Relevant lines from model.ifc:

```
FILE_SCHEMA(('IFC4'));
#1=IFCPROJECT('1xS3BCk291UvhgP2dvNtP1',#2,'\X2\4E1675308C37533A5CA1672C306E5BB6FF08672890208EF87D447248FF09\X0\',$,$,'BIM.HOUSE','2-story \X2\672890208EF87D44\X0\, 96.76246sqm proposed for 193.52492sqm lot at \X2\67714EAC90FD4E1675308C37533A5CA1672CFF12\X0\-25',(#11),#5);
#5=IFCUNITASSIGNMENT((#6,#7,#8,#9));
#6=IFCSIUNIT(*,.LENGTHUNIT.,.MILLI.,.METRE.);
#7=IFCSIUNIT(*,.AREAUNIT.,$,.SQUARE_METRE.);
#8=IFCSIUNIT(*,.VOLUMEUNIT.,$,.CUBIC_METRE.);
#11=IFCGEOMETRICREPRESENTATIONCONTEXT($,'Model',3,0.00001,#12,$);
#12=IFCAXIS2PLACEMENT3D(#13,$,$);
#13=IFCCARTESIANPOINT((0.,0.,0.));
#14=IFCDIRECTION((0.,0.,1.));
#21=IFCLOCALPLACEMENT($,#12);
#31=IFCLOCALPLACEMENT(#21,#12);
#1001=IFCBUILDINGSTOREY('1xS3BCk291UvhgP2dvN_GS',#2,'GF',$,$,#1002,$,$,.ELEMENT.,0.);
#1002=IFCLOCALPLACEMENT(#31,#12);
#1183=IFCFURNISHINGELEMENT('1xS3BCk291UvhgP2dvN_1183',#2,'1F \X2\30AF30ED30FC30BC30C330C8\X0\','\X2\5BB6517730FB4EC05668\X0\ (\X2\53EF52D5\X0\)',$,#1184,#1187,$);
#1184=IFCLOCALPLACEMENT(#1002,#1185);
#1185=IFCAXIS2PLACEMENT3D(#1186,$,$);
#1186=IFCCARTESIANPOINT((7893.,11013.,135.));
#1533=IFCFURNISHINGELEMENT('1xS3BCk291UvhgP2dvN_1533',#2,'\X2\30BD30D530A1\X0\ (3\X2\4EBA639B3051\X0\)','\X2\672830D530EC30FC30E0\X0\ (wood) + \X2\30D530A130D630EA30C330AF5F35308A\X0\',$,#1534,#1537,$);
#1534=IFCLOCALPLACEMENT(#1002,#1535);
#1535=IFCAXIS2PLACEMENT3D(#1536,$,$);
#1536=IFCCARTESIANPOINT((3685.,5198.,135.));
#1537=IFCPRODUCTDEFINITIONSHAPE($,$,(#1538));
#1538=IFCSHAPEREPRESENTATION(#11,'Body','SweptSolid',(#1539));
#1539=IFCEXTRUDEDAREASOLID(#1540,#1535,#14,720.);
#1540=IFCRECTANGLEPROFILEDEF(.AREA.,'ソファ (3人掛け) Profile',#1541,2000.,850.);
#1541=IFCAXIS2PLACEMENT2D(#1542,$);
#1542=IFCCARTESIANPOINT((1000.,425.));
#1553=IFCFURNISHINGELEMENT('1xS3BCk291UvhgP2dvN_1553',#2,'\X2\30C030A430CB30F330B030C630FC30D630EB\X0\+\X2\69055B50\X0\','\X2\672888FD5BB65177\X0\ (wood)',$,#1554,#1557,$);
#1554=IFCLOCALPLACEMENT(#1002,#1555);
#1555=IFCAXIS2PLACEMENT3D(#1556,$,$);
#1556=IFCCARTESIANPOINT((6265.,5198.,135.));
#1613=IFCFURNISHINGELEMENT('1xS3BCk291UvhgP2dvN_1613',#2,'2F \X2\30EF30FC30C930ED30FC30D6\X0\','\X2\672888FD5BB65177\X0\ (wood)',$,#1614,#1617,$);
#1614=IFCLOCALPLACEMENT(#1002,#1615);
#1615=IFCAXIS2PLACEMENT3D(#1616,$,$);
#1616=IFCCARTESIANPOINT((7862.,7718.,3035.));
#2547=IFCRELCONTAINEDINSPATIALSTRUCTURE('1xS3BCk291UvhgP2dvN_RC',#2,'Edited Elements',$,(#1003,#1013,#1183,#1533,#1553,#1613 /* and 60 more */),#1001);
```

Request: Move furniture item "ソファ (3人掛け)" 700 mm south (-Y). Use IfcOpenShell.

```python
import ifcopenshell
import ifcopenshell.api.geometry
import ifcopenshell.util.placement

model = ifcopenshell.open("model.ifc")

item = model.by_guid("1xS3BCk291UvhgP2dvN_1533")
matrix = ifcopenshell.util.placement.get_local_placement(item.ObjectPlacement)
matrix[1, 3] -= 700.0
ifcopenshell.api.geometry.edit_object_placement(model, product=item, matrix=matrix, is_si=False)

print(ifcopenshell.util.placement.get_local_placement(item.ObjectPlacement).round(3) + 0.0)

model.write("model_edited.ifc")
```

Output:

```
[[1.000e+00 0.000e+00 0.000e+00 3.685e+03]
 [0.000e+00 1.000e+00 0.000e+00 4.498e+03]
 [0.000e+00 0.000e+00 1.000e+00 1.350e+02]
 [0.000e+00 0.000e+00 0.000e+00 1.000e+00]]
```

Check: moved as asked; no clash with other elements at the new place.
